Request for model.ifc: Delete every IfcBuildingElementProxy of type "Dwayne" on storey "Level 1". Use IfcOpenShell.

First a look at what the model holds.

```python
import ifcopenshell
import ifcopenshell.util.element

model = ifcopenshell.open("model.ifc")
print(model.schema)
storey = next(s for s in model.by_type("IfcBuildingStorey") if s.Name == "Level 1")
proxies = [e for e in ifcopenshell.util.element.get_decomposition(storey) if e.is_a("IfcBuildingElementProxy")]
seen = {}
for e in proxies:
    element_type = ifcopenshell.util.element.get_type(e)
    name = element_type.Name if element_type not in (None, e) else None
    seen[name] = seen.get(name, 0) + 1
for name, count in sorted(seen.items(), key=str):
    print(count, "x", name)
```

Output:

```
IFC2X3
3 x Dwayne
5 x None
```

```python
import ifcopenshell
import ifcopenshell.api.root
import ifcopenshell.util.element

model = ifcopenshell.open("model.ifc")

storey = next(s for s in model.by_type("IfcBuildingStorey") if s.Name == "Level 1")
proxies = [e for e in ifcopenshell.util.element.get_decomposition(storey) if e.is_a("IfcBuildingElementProxy")]
targets = [e for e in proxies if (t := ifcopenshell.util.element.get_type(e)) not in (None, e) and t.Name == "Dwayne"]

for e in targets:
    ifcopenshell.api.root.remove_product(model, product=e)
print(len(targets), "removed")

model.write("model_v2.ifc")
```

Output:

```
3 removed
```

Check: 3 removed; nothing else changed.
